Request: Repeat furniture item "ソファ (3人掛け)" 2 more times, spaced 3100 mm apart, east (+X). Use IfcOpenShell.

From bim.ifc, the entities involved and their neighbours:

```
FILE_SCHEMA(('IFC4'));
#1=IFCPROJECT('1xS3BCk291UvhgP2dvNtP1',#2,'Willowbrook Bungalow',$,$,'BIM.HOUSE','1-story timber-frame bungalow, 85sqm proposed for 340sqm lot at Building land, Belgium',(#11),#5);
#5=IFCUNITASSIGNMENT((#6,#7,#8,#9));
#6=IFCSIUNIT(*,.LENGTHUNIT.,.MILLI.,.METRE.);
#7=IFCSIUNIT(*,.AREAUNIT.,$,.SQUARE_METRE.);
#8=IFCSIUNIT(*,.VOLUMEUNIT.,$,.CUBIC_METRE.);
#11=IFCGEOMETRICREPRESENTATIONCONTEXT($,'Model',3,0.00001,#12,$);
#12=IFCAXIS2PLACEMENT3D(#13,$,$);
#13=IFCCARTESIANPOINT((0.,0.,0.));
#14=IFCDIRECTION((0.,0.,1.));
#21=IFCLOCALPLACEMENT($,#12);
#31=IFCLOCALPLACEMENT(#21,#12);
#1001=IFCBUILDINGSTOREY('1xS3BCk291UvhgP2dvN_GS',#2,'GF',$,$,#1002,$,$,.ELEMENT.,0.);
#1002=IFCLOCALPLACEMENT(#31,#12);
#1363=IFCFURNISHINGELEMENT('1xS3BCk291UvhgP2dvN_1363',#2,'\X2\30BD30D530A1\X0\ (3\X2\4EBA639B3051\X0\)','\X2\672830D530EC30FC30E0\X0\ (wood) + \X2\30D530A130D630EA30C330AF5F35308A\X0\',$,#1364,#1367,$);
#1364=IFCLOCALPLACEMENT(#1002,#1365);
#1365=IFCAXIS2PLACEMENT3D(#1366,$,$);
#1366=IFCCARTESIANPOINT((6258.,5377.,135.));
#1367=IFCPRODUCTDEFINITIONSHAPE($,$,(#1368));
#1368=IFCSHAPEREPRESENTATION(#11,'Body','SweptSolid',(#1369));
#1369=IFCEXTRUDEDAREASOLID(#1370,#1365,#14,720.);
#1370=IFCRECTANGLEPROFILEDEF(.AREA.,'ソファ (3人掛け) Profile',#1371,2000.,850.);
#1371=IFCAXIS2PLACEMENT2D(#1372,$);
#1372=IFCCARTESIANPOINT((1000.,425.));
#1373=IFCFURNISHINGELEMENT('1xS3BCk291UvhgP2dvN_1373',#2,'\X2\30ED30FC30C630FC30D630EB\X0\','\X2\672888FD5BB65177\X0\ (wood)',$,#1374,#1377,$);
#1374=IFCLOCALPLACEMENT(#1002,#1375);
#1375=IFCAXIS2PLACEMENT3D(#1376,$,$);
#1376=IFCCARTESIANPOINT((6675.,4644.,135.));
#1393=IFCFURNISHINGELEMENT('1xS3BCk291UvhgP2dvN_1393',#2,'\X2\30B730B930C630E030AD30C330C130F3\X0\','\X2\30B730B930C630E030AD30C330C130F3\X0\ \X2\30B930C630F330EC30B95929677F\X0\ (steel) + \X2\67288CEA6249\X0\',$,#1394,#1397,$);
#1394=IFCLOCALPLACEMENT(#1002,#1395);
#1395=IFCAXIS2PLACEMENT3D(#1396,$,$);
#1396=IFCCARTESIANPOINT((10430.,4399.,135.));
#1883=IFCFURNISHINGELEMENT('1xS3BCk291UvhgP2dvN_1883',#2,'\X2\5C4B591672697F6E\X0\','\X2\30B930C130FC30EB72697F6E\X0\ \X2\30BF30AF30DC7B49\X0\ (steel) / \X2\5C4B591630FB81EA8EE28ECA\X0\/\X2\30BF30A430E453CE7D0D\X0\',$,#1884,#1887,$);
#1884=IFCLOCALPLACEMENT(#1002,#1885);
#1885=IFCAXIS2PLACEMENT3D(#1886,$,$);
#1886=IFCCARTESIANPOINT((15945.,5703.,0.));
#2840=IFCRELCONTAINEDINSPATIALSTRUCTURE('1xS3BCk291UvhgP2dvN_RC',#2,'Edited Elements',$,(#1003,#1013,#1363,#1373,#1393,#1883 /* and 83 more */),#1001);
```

```python
import numpy as np
import ifcopenshell
import ifcopenshell.api.geometry
import ifcopenshell.api.root
import ifcopenshell.util.element
import ifcopenshell.util.placement

model = ifcopenshell.open("bim.ifc")


def reuse_history(source, copy):
    """copy_class also copies each property set's owner history, people and application; keep the originals."""
    for rel in copy.IsDefinedBy:
        if rel.is_a("IfcRelDefinesByProperties") and (history := rel.RelatingPropertyDefinition.OwnerHistory):
            rel.RelatingPropertyDefinition.OwnerHistory = source.OwnerHistory
            ifcopenshell.util.element.remove_deep2(model, history)


source = model.by_guid("1xS3BCk291UvhgP2dvN_1363")
base = ifcopenshell.util.placement.get_local_placement(source.ObjectPlacement)
step = np.array([1.0, 0.0, 0.0]) * 3100.0

for i in range(1, 3):
    copy = ifcopenshell.api.root.copy_class(model, product=source)
    copy.Representation = ifcopenshell.util.element.copy_deep(
        model, source.Representation, exclude=["IfcGeometricRepresentationContext", "IfcRepresentationMap"]
    )
    reuse_history(source, copy)
    matrix = base.copy()
    matrix[:3, 3] += i * step
    print("added at", matrix[:3, 3].round(3) + 0.0)
    ifcopenshell.api.geometry.edit_object_placement(model, product=copy, matrix=matrix, is_si=False)

model.write("bim_updated.ifc")
```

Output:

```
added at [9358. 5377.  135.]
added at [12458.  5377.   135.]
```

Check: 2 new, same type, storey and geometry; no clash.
